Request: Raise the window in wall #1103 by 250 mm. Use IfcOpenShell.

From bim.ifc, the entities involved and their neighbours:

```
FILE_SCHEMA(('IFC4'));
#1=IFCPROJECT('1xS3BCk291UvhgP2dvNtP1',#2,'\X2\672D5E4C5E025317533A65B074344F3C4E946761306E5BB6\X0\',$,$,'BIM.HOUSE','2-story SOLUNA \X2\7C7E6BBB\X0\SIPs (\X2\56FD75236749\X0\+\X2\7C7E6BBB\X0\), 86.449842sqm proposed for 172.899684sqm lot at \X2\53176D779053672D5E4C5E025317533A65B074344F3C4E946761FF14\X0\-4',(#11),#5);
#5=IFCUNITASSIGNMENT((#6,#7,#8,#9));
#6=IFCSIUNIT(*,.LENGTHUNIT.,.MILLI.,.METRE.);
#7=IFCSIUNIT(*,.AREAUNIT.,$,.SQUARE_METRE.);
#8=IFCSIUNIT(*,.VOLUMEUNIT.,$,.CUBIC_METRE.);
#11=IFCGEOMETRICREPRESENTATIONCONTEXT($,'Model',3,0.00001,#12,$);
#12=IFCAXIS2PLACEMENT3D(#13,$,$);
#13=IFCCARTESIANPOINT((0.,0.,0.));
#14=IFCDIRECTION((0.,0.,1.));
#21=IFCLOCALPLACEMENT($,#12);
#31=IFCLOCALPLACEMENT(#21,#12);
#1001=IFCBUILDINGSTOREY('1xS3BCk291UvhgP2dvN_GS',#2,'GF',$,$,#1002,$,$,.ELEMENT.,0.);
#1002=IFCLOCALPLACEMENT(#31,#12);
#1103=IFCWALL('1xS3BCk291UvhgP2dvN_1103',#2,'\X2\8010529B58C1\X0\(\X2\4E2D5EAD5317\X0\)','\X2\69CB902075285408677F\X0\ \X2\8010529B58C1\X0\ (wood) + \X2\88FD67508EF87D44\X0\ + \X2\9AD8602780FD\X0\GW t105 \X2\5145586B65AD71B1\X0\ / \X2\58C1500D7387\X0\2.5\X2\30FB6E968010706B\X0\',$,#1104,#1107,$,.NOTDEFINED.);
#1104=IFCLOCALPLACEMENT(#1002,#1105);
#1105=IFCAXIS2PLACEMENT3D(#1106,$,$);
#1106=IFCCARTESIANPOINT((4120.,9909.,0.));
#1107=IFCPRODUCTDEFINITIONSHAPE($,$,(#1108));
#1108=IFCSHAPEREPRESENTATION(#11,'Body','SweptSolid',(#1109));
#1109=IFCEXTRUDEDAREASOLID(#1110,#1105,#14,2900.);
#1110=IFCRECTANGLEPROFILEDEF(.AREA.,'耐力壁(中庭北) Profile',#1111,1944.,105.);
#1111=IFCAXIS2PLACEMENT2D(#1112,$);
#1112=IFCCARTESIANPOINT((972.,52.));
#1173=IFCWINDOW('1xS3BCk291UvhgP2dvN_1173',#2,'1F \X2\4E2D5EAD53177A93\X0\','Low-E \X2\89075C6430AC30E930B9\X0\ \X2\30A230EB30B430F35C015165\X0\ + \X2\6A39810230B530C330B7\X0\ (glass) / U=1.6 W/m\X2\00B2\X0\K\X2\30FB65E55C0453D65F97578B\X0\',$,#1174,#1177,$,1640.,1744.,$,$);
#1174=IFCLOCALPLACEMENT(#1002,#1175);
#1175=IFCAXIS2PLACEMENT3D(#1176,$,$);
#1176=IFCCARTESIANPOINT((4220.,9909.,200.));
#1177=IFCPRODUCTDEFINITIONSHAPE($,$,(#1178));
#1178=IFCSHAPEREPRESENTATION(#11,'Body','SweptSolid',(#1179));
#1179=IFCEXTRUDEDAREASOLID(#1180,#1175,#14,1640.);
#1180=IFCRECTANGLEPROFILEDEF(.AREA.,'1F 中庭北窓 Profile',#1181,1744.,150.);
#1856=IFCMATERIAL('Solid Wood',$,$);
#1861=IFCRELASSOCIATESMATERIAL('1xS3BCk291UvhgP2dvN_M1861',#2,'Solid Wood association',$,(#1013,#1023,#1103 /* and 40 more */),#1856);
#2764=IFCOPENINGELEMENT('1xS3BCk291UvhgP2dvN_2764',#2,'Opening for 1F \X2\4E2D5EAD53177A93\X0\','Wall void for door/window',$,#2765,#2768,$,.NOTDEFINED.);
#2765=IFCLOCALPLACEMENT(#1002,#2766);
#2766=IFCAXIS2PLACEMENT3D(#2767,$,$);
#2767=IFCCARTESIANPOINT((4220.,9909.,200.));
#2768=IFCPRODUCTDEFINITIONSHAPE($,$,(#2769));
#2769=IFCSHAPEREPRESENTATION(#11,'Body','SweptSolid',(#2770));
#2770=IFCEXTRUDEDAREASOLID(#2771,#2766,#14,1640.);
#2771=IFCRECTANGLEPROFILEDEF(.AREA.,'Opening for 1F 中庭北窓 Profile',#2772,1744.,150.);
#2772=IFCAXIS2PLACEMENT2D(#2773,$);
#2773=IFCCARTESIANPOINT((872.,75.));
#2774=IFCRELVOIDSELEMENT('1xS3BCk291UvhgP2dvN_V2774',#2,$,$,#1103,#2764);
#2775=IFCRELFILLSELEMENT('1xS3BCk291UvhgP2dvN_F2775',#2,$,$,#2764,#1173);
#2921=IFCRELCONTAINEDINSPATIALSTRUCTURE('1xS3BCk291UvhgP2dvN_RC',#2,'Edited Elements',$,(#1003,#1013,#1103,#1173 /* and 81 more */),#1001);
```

```python
import numpy as np
import ifcopenshell
import ifcopenshell.api.geometry
import ifcopenshell.util.placement
import ifcopenshell.util.unit

model = ifcopenshell.open("bim.ifc")
unit_scale = ifcopenshell.util.unit.calculate_unit_scale(model)

window = model.by_guid("1xS3BCk291UvhgP2dvN_1173")
opening = window.FillsVoids[0].RelatingOpeningElement
dz = 0.25 / unit_scale

shift = np.array([0.0, 0.0, dz])
# The window is not placed relative to its opening, so move both.
for product in (opening, window):
    matrix = ifcopenshell.util.placement.get_local_placement(product.ObjectPlacement)
    matrix[:3, 3] += shift
    ifcopenshell.api.geometry.edit_object_placement(model, product=product, matrix=matrix, is_si=False)

print(f"moved by {dz * unit_scale:+.3f} m")

model.write("bim_updated.ifc")
```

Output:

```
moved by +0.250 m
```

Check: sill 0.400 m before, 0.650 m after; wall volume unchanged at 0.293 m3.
